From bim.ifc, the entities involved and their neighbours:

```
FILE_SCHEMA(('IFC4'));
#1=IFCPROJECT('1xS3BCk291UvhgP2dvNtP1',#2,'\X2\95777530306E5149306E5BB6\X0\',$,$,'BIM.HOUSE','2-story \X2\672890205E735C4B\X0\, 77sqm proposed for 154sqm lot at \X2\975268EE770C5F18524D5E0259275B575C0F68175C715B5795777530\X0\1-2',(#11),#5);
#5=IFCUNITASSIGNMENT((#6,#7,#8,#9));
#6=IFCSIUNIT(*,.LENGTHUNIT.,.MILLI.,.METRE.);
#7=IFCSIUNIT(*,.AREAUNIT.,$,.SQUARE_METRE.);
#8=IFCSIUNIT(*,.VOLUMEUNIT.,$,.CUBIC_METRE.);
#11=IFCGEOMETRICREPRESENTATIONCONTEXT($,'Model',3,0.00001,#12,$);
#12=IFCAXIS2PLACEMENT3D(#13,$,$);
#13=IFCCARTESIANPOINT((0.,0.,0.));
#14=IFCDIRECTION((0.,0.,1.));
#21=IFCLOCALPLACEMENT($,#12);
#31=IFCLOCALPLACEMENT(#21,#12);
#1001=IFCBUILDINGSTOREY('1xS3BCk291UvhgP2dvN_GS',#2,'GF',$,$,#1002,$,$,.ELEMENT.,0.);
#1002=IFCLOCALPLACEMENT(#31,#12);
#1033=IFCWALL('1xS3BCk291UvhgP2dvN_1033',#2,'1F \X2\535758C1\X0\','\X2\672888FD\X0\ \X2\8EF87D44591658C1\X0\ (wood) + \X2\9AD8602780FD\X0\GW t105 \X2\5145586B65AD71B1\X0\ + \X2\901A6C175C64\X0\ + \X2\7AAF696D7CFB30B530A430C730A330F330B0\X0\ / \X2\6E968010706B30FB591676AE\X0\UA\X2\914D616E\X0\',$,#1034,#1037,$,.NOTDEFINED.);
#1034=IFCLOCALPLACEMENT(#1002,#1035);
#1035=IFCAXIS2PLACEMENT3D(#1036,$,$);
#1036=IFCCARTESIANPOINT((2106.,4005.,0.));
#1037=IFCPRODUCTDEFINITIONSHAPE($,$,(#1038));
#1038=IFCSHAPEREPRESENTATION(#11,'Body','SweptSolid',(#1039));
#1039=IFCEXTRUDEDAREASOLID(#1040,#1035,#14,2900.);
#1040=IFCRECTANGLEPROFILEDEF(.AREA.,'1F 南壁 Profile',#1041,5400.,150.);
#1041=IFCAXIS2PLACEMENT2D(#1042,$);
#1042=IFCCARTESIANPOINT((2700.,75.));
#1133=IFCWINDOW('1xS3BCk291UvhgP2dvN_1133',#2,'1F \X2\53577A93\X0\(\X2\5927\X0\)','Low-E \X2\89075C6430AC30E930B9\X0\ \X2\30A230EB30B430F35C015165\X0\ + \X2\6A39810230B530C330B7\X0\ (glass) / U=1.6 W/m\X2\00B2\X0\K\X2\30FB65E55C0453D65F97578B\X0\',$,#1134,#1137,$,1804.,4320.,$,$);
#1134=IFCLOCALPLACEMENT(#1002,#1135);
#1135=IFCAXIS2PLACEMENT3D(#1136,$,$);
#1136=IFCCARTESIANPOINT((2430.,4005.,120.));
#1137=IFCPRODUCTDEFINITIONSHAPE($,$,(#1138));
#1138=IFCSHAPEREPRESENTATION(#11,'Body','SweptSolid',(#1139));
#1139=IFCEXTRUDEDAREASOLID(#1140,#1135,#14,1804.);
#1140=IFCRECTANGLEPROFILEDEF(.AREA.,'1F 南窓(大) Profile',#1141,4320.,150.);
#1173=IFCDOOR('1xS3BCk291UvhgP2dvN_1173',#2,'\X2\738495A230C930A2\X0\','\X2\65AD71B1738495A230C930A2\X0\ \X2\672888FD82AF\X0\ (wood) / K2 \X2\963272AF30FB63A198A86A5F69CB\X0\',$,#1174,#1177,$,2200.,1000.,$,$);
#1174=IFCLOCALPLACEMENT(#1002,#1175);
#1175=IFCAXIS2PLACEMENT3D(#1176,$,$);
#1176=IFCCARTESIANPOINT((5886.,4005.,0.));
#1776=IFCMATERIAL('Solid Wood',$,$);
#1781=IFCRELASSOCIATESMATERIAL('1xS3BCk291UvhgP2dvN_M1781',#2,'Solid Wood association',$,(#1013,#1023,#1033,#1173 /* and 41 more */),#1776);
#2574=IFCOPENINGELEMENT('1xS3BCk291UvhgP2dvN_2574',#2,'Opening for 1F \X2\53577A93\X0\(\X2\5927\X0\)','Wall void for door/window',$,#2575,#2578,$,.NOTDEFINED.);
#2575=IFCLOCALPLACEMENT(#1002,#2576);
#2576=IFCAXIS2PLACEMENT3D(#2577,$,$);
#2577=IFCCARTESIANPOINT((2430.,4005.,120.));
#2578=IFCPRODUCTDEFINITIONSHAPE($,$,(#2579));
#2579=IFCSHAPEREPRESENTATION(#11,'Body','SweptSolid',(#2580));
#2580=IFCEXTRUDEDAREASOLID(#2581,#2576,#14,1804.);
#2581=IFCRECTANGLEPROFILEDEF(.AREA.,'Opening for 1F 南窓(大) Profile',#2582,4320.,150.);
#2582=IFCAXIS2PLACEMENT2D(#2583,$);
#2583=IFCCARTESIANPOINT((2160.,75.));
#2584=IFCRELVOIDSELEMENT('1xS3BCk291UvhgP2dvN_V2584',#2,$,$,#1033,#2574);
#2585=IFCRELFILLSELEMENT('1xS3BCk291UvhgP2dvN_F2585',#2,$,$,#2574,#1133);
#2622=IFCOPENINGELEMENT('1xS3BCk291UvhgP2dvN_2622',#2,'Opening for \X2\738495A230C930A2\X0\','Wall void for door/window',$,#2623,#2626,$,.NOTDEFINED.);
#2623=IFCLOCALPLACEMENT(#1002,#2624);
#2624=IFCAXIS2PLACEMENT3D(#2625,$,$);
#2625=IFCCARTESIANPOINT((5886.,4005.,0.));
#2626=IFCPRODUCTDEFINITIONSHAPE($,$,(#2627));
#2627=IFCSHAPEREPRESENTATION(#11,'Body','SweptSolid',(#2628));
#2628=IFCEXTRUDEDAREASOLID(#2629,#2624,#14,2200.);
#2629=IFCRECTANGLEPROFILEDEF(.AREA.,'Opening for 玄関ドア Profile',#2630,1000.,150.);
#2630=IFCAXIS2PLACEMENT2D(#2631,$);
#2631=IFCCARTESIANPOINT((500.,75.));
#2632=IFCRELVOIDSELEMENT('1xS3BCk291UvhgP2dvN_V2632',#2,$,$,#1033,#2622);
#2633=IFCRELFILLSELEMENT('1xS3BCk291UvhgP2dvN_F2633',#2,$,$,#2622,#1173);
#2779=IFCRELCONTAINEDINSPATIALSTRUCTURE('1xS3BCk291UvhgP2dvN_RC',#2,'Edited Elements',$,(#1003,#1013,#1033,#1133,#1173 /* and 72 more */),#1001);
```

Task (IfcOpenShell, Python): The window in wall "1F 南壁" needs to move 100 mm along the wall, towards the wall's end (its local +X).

```python
import ifcopenshell
import ifcopenshell.api.geometry
import ifcopenshell.util.placement

model = ifcopenshell.open("bim.ifc")

window = model.by_guid("1xS3BCk291UvhgP2dvN_1133")
opening = window.FillsVoids[0].RelatingOpeningElement
wall = opening.VoidsElements[0].RelatingBuildingElement

wall_matrix = ifcopenshell.util.placement.get_local_placement(wall.ObjectPlacement)
shift = wall_matrix[:3, 0] * 100.0
before = ifcopenshell.util.placement.get_local_placement(window.ObjectPlacement)[:3, 3].copy()

# The window is not placed relative to its opening, so move both.
for product in (opening, window):
    matrix = ifcopenshell.util.placement.get_local_placement(product.ObjectPlacement)
    matrix[:3, 3] += shift
    ifcopenshell.api.geometry.edit_object_placement(model, product=product, matrix=matrix, is_si=False)

after = ifcopenshell.util.placement.get_local_placement(window.ObjectPlacement)[:3, 3]
print("window moved by", (after - before).round(3) + 0.0)

model.write("bim-out.ifc")
```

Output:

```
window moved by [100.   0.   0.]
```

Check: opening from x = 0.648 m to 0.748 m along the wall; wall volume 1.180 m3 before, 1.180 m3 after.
